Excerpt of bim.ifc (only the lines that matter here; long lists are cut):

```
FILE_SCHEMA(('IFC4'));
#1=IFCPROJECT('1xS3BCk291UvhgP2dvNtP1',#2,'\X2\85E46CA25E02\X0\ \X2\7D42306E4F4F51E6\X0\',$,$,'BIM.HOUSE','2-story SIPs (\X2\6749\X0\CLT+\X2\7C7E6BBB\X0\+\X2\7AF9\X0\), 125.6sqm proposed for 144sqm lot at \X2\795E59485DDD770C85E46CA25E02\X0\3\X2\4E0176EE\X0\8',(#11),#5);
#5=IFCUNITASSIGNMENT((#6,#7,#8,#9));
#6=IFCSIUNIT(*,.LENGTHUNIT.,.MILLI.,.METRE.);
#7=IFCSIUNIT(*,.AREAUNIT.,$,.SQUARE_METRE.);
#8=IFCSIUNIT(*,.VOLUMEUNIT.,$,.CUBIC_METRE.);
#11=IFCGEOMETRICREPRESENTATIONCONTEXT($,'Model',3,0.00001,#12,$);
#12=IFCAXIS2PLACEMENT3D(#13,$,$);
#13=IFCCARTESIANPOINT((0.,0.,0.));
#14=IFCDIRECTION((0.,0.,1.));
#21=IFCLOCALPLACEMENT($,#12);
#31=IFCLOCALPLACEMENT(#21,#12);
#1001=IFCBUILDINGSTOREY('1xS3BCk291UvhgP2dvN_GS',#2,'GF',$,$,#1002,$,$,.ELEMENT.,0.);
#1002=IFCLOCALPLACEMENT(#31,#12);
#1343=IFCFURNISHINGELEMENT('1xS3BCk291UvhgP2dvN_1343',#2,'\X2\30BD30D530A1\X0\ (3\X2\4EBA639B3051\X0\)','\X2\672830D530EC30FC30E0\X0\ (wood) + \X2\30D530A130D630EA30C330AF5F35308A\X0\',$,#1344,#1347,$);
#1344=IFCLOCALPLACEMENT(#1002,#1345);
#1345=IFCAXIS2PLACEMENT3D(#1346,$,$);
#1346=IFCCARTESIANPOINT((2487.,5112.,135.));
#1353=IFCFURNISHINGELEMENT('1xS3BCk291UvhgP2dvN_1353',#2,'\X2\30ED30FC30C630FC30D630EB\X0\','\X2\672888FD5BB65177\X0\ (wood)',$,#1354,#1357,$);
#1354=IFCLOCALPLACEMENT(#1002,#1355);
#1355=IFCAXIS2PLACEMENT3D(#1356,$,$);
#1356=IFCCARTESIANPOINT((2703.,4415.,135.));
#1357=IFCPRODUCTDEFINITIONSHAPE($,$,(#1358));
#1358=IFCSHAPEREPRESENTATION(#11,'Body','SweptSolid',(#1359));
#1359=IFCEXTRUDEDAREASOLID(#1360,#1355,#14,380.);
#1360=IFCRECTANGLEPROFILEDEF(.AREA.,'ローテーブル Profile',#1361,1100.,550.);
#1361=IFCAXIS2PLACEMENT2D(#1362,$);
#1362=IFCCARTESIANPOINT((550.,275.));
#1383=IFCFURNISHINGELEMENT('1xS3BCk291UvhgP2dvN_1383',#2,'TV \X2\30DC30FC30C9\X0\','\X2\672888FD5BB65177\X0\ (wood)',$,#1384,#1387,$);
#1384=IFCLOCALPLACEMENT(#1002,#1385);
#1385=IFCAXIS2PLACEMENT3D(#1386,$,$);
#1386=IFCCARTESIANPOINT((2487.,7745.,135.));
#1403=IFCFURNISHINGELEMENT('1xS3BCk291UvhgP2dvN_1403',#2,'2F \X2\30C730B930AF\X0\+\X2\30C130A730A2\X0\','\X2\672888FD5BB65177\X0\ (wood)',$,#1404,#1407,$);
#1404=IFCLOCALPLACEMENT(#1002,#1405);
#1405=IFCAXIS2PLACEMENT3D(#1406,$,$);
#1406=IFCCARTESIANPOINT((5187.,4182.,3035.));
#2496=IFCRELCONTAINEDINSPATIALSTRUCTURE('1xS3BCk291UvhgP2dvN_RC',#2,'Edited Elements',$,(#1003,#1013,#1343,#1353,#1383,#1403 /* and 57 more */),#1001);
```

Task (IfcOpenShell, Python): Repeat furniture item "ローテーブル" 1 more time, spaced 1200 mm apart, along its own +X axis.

```python
import ifcopenshell
import ifcopenshell.api.geometry
import ifcopenshell.api.root
import ifcopenshell.util.element
import ifcopenshell.util.placement
import ifcopenshell.util.unit

model = ifcopenshell.open("bim.ifc")
unit_scale = ifcopenshell.util.unit.calculate_unit_scale(model)


def reuse_history(source, copy):
    """copy_class also copies each property set's owner history, people and application; keep the originals."""
    for rel in copy.IsDefinedBy:
        if rel.is_a("IfcRelDefinesByProperties") and (history := rel.RelatingPropertyDefinition.OwnerHistory):
            rel.RelatingPropertyDefinition.OwnerHistory = source.OwnerHistory
            ifcopenshell.util.element.remove_deep2(model, history)


source = model.by_guid("1xS3BCk291UvhgP2dvN_1353")
base = ifcopenshell.util.placement.get_local_placement(source.ObjectPlacement)
step = base[:3, 0] * 1.2 / unit_scale

for i in range(1, 2):
    copy = ifcopenshell.api.root.copy_class(model, product=source)
    copy.Representation = ifcopenshell.util.element.copy_deep(
        model, source.Representation, exclude=["IfcGeometricRepresentationContext", "IfcRepresentationMap"]
    )
    reuse_history(source, copy)
    matrix = base.copy()
    matrix[:3, 3] += i * step
    print("added at", matrix[:3, 3].round(3) + 0.0)
    ifcopenshell.api.geometry.edit_object_placement(model, product=copy, matrix=matrix, is_si=False)

model.write("bim_v2.ifc")
```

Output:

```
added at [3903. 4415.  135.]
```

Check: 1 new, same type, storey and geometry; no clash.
